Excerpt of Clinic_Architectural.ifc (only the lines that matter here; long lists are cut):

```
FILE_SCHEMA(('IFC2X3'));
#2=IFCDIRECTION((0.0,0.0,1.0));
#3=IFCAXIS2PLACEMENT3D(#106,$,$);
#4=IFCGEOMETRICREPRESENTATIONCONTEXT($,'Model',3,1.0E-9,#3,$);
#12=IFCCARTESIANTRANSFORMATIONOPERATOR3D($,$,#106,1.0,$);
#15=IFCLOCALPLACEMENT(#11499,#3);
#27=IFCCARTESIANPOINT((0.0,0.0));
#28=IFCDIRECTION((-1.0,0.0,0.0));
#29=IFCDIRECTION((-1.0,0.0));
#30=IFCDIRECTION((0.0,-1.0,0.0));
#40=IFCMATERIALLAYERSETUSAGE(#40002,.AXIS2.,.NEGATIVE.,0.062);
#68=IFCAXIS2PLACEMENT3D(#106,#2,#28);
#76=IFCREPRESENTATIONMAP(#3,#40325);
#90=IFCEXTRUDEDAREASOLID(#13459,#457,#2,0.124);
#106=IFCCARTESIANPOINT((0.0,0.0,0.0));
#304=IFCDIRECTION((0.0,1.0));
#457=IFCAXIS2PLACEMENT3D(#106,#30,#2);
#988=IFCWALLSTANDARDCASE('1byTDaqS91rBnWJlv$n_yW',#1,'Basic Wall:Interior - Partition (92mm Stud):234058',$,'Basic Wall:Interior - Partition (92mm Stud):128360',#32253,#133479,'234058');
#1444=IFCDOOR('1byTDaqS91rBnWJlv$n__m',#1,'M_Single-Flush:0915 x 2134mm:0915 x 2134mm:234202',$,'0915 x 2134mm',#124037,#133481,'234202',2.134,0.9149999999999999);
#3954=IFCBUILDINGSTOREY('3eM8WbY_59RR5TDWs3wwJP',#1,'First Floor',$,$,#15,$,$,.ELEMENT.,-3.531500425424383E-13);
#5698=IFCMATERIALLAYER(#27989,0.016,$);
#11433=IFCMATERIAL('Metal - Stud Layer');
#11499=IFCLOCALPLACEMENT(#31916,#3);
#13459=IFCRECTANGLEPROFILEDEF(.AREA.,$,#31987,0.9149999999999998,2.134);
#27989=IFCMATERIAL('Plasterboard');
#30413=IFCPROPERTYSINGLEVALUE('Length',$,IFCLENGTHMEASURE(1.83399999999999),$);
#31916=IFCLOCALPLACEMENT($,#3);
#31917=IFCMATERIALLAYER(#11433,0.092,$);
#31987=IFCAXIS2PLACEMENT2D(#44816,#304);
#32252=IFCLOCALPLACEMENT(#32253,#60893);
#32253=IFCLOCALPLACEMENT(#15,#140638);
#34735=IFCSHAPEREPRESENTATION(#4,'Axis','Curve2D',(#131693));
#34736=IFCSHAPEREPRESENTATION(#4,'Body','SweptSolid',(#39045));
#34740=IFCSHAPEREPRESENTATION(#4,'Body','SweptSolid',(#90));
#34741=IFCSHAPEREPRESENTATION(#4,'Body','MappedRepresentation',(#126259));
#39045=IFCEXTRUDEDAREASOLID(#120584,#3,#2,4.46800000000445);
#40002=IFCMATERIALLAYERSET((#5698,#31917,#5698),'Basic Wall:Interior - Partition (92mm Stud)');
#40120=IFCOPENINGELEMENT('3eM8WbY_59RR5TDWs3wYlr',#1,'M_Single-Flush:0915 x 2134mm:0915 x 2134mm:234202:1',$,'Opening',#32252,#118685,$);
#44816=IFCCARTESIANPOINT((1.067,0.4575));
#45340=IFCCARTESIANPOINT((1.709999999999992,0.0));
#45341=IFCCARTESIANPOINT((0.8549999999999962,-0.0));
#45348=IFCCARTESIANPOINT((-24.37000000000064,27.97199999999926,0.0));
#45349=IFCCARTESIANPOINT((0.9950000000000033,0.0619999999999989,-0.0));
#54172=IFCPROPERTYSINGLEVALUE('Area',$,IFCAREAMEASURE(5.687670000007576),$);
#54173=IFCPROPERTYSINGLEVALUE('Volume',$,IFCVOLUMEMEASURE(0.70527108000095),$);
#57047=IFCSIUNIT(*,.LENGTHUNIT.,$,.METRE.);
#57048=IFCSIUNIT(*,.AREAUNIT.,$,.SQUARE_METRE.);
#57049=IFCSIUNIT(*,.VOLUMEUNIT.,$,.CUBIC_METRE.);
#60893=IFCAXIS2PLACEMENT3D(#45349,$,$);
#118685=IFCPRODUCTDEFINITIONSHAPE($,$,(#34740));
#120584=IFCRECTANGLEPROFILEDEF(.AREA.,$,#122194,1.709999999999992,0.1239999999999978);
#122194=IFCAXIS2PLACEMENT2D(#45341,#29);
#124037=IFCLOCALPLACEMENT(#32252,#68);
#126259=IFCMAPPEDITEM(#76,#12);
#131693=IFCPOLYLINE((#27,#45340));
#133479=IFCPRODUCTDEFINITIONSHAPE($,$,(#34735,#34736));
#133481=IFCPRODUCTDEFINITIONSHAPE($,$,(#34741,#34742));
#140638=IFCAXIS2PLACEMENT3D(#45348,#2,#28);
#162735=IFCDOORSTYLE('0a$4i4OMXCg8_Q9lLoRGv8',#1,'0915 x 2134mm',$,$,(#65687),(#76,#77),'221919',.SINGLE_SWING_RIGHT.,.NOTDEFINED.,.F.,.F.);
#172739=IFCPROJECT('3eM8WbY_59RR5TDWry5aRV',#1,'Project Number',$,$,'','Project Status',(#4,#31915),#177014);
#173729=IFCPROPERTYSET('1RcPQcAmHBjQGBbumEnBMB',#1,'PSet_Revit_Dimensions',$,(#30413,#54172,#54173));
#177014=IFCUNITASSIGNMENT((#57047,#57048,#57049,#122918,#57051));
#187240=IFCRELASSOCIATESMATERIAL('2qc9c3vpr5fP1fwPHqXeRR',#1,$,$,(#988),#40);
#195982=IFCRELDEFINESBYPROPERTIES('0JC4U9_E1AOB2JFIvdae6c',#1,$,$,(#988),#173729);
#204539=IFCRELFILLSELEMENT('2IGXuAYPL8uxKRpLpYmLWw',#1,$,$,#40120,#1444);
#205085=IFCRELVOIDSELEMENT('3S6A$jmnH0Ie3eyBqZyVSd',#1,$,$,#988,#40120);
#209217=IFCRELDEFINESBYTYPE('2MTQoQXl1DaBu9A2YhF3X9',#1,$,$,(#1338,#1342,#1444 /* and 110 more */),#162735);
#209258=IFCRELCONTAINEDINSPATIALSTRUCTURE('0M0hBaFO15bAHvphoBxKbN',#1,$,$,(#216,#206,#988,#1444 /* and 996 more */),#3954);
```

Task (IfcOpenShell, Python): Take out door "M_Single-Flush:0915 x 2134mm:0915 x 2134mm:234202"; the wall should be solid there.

```python
import ifcopenshell
import ifcopenshell.api.feature
import ifcopenshell.api.pset
import ifcopenshell.api.root
import ifcopenshell.geom
import ifcopenshell.util.element
import ifcopenshell.util.shape
import ifcopenshell.util.unit

model = ifcopenshell.open("Clinic_Architectural.ifc")
area_scale = ifcopenshell.util.unit.calculate_unit_scale(model, "AREAUNIT")
volume_scale = ifcopenshell.util.unit.calculate_unit_scale(model, "VOLUMEUNIT")
settings = ifcopenshell.geom.settings()


def volume(element):
    """Net volume in cubic metres, openings subtracted."""
    shape = ifcopenshell.geom.create_shape(settings, element)
    return ifcopenshell.util.shape.get_volume(shape.geometry)


door = model.by_guid("1byTDaqS91rBnWJlv$n__m")
opening = door.FillsVoids[0].RelatingOpeningElement
wall = opening.VoidsElements[0].RelatingBuildingElement
before = volume(wall)

ifcopenshell.api.root.remove_product(model, product=door)
ifcopenshell.api.feature.remove_feature(model, feature=opening)

after = volume(wall)
thickness = 0.124  # wall thickness in metres

# Update the wall's stored quantities.
pset = model.by_id(ifcopenshell.util.element.get_pset(wall, "PSet_Revit_Dimensions", should_inherit=False)["id"])
ifcopenshell.api.pset.edit_pset(model, pset=pset, properties={
    "Area": model.create_entity("IfcAreaMeasure", after / thickness / area_scale),
    "Volume": model.create_entity("IfcVolumeMeasure", after / volume_scale),
})

print(f"wall volume {before:.3f} -> {after:.3f} m3")

model.write("Clinic_Architectural_updated.ifc")
```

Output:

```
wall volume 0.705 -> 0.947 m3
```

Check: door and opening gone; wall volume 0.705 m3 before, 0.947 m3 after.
